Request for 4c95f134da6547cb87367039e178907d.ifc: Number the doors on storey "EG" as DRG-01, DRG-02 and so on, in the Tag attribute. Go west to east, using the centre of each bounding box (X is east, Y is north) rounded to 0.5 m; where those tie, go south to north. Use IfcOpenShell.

First a look at what the model holds.

```python
import ifcopenshell
import ifcopenshell.util.element
import ifcopenshell.util.placement

model = ifcopenshell.open("4c95f134da6547cb87367039e178907d.ifc")
print(model.schema)
storey = next(s for s in model.by_type("IfcBuildingStorey") if s.Name == "EG")
doors = [e for e in ifcopenshell.util.element.get_decomposition(storey) if e.is_a("IfcDoor")]
for e in sorted(doors, key=lambda e: e.id()):
    origin = ifcopenshell.util.placement.get_local_placement(e.ObjectPlacement)[:3, 3]
    print(e.id(), e.Tag, e.Name, origin.round(2) + 0.0, sep=" | ")
```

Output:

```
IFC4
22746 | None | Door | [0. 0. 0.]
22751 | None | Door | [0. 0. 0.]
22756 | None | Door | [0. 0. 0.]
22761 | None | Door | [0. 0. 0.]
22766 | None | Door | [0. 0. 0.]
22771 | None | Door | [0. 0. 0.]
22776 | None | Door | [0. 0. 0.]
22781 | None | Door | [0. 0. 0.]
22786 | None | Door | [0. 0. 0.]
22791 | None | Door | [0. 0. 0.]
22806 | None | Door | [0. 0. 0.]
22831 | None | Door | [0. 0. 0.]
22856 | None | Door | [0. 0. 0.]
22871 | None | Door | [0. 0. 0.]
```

```python
import ifcopenshell
import ifcopenshell.geom
import ifcopenshell.util.element
import ifcopenshell.util.shape

model = ifcopenshell.open("4c95f134da6547cb87367039e178907d.ifc")
settings = ifcopenshell.geom.settings()
settings.set("use-world-coords", True)


def centre(element):
    shape = ifcopenshell.geom.create_shape(settings, element)
    return ifcopenshell.util.shape.get_bbox_centroid(shape.geometry)


storey = next(s for s in model.by_type("IfcBuildingStorey") if s.Name == "EG")
doors = [e for e in ifcopenshell.util.element.get_decomposition(storey) if e.is_a("IfcDoor")]

# Insertion points can sit at a corner or the storey origin, so sort by the geometry (in metres).
centres = {e: centre(e) for e in doors}
doors.sort(key=lambda e: (round(centres[e][0] / 0.5), centres[e][1]))

for i, e in enumerate(doors, start=1):
    number = f"DRG-{i:02d}"
    e.Tag = number
    print(e.id(), number)

model.write("4c95f134da6547cb87367039e178907d_edited.ifc")
```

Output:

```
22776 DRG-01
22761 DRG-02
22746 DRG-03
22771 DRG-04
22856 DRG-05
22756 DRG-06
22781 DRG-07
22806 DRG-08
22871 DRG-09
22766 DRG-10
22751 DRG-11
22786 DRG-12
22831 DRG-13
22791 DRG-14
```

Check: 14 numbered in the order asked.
